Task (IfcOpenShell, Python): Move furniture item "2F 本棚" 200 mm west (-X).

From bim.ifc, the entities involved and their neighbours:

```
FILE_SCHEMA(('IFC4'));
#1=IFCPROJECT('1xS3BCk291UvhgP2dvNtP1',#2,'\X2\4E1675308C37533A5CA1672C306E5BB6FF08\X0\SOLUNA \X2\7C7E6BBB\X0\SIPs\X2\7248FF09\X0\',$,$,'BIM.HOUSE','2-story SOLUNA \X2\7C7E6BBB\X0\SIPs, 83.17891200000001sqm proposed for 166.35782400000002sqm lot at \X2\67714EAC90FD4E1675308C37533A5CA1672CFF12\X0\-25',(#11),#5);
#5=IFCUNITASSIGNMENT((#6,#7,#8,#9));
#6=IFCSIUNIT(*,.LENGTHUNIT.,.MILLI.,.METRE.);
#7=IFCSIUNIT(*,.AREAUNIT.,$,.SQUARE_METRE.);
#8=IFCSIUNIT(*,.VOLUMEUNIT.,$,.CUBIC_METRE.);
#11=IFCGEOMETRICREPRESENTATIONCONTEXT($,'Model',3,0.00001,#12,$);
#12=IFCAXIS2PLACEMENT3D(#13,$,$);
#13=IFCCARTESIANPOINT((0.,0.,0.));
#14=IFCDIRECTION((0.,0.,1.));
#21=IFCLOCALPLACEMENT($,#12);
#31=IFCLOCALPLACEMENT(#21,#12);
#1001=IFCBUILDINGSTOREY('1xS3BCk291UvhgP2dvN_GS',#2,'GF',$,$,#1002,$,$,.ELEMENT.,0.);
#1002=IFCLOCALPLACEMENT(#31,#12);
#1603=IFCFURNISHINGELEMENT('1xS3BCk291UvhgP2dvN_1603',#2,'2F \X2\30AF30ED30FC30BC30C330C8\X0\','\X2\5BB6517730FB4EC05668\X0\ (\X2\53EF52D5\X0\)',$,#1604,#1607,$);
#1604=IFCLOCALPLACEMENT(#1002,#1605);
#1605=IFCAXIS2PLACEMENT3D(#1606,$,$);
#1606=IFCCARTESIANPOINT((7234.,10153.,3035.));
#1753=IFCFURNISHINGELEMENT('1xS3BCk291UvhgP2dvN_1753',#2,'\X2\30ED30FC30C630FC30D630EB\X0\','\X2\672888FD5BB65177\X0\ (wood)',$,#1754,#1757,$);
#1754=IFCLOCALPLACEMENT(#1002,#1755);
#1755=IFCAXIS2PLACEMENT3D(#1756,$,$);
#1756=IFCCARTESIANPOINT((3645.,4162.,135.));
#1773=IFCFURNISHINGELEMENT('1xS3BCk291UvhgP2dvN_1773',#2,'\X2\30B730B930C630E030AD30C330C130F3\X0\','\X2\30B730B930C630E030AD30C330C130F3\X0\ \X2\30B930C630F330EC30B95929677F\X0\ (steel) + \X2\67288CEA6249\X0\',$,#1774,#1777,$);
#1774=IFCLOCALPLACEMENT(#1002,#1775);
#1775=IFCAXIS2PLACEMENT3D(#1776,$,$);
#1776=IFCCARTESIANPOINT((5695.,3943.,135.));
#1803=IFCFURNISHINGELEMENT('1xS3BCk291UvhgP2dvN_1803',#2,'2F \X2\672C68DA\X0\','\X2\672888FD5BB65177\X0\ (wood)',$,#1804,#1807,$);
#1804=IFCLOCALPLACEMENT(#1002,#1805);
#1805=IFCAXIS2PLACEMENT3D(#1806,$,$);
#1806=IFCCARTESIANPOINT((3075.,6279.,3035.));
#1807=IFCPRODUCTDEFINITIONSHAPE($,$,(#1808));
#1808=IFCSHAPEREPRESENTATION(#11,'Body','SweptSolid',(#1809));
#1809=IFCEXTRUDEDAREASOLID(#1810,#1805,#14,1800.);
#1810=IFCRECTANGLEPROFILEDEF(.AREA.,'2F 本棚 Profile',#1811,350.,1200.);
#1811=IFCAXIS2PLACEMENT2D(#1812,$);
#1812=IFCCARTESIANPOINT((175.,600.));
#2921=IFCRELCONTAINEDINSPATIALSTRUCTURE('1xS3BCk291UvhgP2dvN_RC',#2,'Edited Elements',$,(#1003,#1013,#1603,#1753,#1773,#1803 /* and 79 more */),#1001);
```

```python
import ifcopenshell
import ifcopenshell.api.geometry
import ifcopenshell.util.placement
import ifcopenshell.util.unit

model = ifcopenshell.open("bim.ifc")
unit_scale = ifcopenshell.util.unit.calculate_unit_scale(model)

item = model.by_id(1803)
matrix = ifcopenshell.util.placement.get_local_placement(item.ObjectPlacement)
matrix[0, 3] -= 0.2 / unit_scale
ifcopenshell.api.geometry.edit_object_placement(model, product=item, matrix=matrix, is_si=False)

print(ifcopenshell.util.placement.get_local_placement(item.ObjectPlacement).round(3) + 0.0)

model.write("bim-out.ifc")
```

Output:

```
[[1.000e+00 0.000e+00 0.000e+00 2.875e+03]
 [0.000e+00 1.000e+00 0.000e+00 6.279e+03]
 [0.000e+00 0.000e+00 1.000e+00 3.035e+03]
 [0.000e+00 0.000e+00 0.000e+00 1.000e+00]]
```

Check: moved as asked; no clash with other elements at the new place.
